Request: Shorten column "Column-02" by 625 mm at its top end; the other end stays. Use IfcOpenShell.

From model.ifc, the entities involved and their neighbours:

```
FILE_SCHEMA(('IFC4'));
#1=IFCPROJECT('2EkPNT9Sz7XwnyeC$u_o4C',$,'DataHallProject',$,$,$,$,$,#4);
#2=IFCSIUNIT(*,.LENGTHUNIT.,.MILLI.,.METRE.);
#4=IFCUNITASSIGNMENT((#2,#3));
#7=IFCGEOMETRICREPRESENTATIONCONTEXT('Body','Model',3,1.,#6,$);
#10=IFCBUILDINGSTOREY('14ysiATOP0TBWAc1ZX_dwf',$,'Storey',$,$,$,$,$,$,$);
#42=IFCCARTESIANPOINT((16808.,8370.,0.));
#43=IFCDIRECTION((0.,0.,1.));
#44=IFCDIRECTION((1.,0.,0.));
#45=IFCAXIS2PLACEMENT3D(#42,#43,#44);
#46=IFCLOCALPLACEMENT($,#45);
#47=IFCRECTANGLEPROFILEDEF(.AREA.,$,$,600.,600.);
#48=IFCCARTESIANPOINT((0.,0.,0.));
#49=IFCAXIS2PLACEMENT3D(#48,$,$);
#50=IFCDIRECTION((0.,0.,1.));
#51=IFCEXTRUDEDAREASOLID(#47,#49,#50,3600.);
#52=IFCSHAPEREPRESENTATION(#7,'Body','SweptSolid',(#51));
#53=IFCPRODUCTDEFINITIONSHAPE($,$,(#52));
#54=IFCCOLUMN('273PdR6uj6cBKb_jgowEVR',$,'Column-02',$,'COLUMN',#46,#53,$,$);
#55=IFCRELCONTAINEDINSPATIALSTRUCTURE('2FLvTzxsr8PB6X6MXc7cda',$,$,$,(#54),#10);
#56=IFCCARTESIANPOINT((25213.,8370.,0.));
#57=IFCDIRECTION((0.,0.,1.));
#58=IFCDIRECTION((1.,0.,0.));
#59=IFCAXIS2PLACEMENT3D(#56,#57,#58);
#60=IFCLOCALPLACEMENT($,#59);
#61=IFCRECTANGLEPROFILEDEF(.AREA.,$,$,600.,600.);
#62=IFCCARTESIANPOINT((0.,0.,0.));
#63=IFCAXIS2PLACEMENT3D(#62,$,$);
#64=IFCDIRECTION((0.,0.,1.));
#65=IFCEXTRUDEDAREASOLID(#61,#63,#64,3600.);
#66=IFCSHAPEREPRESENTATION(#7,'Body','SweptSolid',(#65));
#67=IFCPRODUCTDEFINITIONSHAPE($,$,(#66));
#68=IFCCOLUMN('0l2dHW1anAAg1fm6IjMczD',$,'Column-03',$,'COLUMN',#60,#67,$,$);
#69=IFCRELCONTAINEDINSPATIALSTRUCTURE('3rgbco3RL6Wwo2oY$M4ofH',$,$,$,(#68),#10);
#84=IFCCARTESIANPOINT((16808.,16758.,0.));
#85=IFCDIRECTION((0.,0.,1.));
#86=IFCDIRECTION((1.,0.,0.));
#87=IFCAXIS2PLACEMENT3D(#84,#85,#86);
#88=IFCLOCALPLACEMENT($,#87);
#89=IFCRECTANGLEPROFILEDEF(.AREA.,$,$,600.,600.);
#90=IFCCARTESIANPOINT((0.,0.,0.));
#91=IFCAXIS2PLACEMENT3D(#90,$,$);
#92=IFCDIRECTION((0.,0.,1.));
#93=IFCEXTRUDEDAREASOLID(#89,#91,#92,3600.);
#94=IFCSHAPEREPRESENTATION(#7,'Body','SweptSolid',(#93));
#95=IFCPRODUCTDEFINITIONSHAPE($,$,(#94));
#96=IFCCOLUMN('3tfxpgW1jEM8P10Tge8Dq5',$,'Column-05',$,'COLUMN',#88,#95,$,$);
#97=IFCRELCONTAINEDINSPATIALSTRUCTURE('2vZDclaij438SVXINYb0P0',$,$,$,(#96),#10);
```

```python
import ifcopenshell

model = ifcopenshell.open("model.ifc")

member = model.by_guid("273PdR6uj6cBKb_jgowEVR")
change = -625.0

# The extrusion runs towards the end named, so only its depth changes.
body = next(r for r in member.Representation.Representations if r.RepresentationIdentifier == "Body")
solid = body.Items[0]
old_length = solid.Depth
solid.Depth += change

print(f"length {old_length:g} -> {solid.Depth:g}")

model.write("model_edited.ifc")
```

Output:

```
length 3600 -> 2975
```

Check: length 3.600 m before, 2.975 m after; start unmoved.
